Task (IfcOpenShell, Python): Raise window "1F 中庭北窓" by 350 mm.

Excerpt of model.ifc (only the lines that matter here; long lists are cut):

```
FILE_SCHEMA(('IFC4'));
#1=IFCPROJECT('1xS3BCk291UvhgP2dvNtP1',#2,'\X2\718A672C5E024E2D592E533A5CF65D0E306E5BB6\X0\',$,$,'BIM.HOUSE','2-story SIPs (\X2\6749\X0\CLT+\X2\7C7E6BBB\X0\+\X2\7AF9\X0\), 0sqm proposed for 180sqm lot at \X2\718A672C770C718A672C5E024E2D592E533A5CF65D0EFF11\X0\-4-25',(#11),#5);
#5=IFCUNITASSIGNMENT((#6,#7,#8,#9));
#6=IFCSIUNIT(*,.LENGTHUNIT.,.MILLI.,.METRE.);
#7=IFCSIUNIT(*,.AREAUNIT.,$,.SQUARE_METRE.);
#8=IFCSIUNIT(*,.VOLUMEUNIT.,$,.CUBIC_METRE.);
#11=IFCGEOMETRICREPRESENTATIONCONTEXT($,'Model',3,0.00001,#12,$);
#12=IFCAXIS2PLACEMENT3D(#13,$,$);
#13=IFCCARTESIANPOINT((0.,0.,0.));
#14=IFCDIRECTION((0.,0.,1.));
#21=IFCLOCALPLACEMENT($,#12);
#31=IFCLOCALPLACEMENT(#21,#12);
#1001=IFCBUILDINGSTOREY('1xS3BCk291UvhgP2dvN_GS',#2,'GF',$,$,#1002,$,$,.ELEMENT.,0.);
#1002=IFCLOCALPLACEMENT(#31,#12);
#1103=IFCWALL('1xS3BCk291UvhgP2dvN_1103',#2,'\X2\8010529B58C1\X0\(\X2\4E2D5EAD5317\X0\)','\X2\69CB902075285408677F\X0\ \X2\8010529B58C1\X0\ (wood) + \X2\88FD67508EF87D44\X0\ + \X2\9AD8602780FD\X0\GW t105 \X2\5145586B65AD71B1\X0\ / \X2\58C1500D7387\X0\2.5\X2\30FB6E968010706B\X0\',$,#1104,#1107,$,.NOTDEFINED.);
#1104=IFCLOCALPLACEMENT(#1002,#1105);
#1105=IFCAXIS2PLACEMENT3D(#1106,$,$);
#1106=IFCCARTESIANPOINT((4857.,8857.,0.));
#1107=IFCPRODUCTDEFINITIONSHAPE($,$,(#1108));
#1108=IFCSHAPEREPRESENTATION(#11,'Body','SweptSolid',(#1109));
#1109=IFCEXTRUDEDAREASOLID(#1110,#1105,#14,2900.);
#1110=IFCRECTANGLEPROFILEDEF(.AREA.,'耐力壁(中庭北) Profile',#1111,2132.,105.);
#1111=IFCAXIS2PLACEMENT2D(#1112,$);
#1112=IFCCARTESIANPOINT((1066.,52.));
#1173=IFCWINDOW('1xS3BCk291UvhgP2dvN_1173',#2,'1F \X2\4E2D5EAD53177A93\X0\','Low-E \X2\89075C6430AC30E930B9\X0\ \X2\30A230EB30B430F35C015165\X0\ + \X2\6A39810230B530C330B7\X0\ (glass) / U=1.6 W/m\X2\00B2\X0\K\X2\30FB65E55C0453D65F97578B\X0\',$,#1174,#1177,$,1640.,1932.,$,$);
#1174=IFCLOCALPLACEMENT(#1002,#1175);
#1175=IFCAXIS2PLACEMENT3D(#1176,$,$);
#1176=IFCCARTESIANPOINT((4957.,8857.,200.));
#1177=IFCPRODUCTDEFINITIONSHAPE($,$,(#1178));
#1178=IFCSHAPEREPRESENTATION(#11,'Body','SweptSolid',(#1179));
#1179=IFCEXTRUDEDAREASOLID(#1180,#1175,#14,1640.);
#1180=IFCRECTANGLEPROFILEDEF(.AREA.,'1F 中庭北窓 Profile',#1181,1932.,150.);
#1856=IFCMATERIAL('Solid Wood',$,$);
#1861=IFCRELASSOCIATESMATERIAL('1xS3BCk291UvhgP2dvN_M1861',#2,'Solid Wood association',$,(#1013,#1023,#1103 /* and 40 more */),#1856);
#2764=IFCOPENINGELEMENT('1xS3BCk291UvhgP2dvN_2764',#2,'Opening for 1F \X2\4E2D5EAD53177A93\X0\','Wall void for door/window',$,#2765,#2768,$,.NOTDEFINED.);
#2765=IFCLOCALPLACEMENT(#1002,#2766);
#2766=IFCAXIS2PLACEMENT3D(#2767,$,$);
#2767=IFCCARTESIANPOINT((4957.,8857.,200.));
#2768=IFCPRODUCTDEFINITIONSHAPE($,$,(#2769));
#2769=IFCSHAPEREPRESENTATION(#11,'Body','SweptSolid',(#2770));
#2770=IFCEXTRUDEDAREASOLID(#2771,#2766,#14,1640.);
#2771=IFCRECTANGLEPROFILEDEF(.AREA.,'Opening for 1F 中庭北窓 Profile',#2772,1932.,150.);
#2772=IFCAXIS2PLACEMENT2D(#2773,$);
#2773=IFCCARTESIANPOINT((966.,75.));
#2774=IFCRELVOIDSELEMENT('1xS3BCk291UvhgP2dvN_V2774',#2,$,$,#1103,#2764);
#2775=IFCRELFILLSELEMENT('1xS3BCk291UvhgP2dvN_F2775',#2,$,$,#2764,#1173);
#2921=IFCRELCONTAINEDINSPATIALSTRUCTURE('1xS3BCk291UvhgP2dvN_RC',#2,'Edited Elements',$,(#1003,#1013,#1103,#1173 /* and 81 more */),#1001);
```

```python
import numpy as np
import ifcopenshell
import ifcopenshell.api.geometry
import ifcopenshell.util.placement
import ifcopenshell.util.unit

model = ifcopenshell.open("model.ifc")
unit_scale = ifcopenshell.util.unit.calculate_unit_scale(model)

window = model.by_guid("1xS3BCk291UvhgP2dvN_1173")
opening = window.FillsVoids[0].RelatingOpeningElement
dz = 350.0

shift = np.array([0.0, 0.0, dz])
# The window is not placed relative to its opening, so move both.
for product in (opening, window):
    matrix = ifcopenshell.util.placement.get_local_placement(product.ObjectPlacement)
    matrix[:3, 3] += shift
    ifcopenshell.api.geometry.edit_object_placement(model, product=product, matrix=matrix, is_si=False)

print(f"moved by {dz * unit_scale:+.3f} m")

model.write("model_updated.ifc")
```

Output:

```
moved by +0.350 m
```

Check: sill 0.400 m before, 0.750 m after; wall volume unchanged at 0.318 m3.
